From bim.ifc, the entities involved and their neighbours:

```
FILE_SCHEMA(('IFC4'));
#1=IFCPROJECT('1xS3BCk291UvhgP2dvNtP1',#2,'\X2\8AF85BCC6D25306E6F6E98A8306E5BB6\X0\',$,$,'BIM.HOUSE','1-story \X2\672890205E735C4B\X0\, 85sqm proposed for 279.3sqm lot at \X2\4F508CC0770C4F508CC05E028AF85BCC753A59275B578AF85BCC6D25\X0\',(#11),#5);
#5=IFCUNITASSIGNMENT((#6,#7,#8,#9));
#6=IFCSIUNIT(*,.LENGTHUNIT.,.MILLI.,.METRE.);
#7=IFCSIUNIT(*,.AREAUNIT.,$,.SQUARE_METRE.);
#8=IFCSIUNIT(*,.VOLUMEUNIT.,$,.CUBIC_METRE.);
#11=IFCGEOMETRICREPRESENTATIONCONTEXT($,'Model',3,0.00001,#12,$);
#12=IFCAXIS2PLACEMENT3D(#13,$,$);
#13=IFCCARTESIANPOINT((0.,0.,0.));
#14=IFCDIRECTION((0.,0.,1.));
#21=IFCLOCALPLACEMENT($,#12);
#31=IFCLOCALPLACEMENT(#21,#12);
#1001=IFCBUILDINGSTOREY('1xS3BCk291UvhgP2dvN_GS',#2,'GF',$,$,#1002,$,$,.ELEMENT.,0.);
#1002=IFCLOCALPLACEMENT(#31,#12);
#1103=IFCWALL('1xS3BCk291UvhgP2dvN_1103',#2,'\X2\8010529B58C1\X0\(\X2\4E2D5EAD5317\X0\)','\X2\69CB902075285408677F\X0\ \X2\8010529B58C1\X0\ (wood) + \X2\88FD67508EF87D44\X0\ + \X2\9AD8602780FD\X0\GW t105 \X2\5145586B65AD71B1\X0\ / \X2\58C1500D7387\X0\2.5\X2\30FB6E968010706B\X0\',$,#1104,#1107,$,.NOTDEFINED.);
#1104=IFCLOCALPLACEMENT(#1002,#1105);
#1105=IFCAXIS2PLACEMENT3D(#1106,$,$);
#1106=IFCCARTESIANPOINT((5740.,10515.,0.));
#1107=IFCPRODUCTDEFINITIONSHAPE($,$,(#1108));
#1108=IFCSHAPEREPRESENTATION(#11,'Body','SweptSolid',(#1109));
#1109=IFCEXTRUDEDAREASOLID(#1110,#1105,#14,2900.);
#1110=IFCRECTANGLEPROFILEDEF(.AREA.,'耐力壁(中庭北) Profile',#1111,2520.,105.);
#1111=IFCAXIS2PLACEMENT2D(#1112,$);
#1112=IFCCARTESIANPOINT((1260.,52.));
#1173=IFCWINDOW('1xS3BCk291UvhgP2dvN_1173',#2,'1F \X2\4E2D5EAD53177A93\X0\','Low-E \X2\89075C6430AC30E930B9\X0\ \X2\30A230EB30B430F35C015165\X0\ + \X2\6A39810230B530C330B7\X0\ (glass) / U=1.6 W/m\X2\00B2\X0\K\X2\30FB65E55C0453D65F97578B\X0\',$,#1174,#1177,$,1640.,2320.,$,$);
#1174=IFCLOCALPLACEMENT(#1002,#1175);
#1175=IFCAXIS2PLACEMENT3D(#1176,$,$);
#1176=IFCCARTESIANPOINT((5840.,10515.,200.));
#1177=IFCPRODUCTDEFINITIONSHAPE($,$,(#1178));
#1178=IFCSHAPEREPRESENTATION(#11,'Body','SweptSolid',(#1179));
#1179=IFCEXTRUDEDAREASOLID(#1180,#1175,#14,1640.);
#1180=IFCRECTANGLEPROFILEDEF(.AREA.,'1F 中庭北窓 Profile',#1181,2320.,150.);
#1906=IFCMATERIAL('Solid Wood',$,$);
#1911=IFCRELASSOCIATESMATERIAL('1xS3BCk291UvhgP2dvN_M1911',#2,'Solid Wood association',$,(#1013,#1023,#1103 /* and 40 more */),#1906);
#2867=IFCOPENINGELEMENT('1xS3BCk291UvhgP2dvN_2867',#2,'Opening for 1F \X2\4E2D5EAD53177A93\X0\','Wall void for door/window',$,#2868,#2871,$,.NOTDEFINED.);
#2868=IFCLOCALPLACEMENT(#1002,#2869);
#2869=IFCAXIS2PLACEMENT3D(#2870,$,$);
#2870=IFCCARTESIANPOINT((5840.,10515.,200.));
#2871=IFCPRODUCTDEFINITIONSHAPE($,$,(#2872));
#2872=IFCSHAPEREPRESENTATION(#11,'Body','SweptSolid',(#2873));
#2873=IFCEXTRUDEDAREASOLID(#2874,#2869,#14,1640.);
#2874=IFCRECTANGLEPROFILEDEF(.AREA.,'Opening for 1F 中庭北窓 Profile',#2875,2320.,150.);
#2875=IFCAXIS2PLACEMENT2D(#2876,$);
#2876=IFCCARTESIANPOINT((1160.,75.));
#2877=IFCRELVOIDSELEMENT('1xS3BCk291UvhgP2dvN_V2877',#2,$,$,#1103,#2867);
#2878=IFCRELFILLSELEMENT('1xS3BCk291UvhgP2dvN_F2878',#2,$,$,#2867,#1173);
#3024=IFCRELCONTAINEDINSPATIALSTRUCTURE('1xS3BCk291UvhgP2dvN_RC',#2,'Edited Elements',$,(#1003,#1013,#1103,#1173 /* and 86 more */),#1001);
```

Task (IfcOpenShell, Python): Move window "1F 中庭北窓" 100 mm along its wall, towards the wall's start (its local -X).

```python
import ifcopenshell
import ifcopenshell.api.geometry
import ifcopenshell.util.placement
import ifcopenshell.util.unit

model = ifcopenshell.open("bim.ifc")
unit_scale = ifcopenshell.util.unit.calculate_unit_scale(model)

window = model.by_guid("1xS3BCk291UvhgP2dvN_1173")
opening = window.FillsVoids[0].RelatingOpeningElement
wall = opening.VoidsElements[0].RelatingBuildingElement

wall_matrix = ifcopenshell.util.placement.get_local_placement(wall.ObjectPlacement)
shift = wall_matrix[:3, 0] * -0.1 / unit_scale
before = ifcopenshell.util.placement.get_local_placement(window.ObjectPlacement)[:3, 3].copy()

# The window is not placed relative to its opening, so move both.
for product in (opening, window):
    matrix = ifcopenshell.util.placement.get_local_placement(product.ObjectPlacement)
    matrix[:3, 3] += shift
    ifcopenshell.api.geometry.edit_object_placement(model, product=product, matrix=matrix, is_si=False)

after = ifcopenshell.util.placement.get_local_placement(window.ObjectPlacement)[:3, 3]
print("window moved by", (after - before).round(3) + 0.0)

model.write("bim_v2.ifc")
```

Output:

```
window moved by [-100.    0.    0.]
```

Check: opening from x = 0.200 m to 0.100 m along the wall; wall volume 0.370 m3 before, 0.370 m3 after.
